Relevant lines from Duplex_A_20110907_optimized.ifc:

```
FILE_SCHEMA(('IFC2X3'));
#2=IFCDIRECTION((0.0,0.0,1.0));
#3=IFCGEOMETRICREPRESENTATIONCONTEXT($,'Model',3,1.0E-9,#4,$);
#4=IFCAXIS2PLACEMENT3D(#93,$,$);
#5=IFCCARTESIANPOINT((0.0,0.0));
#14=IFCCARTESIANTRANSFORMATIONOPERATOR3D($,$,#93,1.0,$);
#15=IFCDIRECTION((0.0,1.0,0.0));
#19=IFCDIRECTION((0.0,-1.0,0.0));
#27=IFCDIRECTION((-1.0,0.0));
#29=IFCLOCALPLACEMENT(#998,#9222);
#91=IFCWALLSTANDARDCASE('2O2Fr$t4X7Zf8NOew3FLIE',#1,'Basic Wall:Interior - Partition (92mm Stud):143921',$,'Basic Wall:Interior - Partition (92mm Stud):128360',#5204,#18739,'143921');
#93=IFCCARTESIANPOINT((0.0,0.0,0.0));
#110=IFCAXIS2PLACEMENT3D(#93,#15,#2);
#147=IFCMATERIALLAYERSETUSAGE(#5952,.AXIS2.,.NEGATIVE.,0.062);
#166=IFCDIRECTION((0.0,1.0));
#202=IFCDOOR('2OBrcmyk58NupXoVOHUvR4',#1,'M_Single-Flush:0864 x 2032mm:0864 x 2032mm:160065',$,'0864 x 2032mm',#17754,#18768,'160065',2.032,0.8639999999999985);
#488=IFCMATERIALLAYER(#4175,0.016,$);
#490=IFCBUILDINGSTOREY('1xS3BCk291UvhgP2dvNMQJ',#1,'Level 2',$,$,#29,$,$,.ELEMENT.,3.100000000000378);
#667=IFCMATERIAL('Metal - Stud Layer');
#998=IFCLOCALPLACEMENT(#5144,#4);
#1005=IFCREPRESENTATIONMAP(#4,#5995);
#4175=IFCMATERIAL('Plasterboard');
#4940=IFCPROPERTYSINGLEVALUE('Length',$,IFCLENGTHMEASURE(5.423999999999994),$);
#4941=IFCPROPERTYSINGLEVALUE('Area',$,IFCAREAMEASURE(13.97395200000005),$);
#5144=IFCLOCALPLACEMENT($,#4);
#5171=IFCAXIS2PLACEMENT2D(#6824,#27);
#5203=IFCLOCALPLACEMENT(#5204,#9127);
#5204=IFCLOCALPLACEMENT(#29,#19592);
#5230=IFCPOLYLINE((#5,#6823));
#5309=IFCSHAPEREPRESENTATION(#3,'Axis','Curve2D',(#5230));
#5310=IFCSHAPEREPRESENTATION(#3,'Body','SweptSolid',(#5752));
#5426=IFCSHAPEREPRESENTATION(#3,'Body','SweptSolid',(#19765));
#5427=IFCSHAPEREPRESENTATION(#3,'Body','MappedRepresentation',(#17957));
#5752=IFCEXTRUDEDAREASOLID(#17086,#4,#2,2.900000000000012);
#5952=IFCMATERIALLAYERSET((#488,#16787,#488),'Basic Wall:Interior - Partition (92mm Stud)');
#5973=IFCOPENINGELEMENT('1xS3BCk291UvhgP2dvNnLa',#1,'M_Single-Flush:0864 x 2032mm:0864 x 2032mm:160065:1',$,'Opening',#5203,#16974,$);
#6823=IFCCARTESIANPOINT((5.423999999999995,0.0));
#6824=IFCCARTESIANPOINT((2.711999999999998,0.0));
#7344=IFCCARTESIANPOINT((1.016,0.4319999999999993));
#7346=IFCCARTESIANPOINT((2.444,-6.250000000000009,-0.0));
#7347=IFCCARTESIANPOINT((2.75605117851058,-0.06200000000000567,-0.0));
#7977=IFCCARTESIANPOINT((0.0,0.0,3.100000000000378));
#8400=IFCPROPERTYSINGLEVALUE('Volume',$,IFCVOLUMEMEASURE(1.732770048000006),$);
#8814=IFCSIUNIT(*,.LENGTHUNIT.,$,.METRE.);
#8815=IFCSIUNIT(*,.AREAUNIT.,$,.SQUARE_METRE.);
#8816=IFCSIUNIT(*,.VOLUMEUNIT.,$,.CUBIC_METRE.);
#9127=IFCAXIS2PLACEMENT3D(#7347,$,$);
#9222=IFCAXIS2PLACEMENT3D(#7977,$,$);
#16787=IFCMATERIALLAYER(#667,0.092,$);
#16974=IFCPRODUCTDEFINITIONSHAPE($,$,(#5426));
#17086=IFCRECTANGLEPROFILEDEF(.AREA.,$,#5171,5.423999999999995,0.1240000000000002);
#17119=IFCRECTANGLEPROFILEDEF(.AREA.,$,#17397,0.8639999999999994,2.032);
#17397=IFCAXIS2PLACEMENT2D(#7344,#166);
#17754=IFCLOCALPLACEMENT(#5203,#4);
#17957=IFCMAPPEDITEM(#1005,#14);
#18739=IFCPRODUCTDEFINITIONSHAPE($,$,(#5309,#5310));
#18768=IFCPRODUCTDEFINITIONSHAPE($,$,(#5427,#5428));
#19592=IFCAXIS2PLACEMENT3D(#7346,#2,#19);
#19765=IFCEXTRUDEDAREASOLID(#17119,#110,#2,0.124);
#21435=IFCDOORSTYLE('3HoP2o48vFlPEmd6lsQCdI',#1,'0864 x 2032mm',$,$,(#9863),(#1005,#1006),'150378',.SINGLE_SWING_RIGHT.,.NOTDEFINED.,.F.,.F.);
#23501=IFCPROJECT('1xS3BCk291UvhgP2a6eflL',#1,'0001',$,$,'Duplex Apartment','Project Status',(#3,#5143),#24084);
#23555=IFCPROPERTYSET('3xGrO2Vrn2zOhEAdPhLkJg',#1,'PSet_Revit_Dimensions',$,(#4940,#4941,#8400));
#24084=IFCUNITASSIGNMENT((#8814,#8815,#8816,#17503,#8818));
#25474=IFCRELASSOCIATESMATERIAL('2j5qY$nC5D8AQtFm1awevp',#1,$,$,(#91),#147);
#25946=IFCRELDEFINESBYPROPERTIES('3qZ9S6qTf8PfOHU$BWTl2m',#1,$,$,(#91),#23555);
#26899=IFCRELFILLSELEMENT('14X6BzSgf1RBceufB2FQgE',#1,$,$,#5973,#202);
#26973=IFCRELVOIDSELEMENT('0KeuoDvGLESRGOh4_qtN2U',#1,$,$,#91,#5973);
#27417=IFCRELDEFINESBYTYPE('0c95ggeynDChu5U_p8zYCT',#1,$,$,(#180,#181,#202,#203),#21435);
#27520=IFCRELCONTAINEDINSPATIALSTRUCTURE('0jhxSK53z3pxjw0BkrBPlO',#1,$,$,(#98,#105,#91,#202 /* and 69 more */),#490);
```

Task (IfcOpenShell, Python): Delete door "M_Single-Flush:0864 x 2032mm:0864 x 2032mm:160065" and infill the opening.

```python
import ifcopenshell
import ifcopenshell.api.feature
import ifcopenshell.api.pset
import ifcopenshell.api.root
import ifcopenshell.geom
import ifcopenshell.util.element
import ifcopenshell.util.shape
import ifcopenshell.util.unit

model = ifcopenshell.open("Duplex_A_20110907_optimized.ifc")
area_scale = ifcopenshell.util.unit.calculate_unit_scale(model, "AREAUNIT")
volume_scale = ifcopenshell.util.unit.calculate_unit_scale(model, "VOLUMEUNIT")
settings = ifcopenshell.geom.settings()


def volume(element):
    """Net volume in cubic metres, openings subtracted."""
    shape = ifcopenshell.geom.create_shape(settings, element)
    return ifcopenshell.util.shape.get_volume(shape.geometry)


door = model.by_guid("2OBrcmyk58NupXoVOHUvR4")
opening = door.FillsVoids[0].RelatingOpeningElement
wall = opening.VoidsElements[0].RelatingBuildingElement
before = volume(wall)

ifcopenshell.api.root.remove_product(model, product=door)
ifcopenshell.api.feature.remove_feature(model, feature=opening)

after = volume(wall)
thickness = 0.124  # wall thickness in metres

# Update the wall's stored quantities.
pset = model.by_id(ifcopenshell.util.element.get_pset(wall, "PSet_Revit_Dimensions", should_inherit=False)["id"])
ifcopenshell.api.pset.edit_pset(model, pset=pset, properties={
    "Area": model.create_entity("IfcAreaMeasure", after / thickness / area_scale),
    "Volume": model.create_entity("IfcVolumeMeasure", after / volume_scale),
})

print(f"wall volume {before:.3f} -> {after:.3f} m3")

model.write("Duplex_A_20110907_optimized_v2.ifc")
```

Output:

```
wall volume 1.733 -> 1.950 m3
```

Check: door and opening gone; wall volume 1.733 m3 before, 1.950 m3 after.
